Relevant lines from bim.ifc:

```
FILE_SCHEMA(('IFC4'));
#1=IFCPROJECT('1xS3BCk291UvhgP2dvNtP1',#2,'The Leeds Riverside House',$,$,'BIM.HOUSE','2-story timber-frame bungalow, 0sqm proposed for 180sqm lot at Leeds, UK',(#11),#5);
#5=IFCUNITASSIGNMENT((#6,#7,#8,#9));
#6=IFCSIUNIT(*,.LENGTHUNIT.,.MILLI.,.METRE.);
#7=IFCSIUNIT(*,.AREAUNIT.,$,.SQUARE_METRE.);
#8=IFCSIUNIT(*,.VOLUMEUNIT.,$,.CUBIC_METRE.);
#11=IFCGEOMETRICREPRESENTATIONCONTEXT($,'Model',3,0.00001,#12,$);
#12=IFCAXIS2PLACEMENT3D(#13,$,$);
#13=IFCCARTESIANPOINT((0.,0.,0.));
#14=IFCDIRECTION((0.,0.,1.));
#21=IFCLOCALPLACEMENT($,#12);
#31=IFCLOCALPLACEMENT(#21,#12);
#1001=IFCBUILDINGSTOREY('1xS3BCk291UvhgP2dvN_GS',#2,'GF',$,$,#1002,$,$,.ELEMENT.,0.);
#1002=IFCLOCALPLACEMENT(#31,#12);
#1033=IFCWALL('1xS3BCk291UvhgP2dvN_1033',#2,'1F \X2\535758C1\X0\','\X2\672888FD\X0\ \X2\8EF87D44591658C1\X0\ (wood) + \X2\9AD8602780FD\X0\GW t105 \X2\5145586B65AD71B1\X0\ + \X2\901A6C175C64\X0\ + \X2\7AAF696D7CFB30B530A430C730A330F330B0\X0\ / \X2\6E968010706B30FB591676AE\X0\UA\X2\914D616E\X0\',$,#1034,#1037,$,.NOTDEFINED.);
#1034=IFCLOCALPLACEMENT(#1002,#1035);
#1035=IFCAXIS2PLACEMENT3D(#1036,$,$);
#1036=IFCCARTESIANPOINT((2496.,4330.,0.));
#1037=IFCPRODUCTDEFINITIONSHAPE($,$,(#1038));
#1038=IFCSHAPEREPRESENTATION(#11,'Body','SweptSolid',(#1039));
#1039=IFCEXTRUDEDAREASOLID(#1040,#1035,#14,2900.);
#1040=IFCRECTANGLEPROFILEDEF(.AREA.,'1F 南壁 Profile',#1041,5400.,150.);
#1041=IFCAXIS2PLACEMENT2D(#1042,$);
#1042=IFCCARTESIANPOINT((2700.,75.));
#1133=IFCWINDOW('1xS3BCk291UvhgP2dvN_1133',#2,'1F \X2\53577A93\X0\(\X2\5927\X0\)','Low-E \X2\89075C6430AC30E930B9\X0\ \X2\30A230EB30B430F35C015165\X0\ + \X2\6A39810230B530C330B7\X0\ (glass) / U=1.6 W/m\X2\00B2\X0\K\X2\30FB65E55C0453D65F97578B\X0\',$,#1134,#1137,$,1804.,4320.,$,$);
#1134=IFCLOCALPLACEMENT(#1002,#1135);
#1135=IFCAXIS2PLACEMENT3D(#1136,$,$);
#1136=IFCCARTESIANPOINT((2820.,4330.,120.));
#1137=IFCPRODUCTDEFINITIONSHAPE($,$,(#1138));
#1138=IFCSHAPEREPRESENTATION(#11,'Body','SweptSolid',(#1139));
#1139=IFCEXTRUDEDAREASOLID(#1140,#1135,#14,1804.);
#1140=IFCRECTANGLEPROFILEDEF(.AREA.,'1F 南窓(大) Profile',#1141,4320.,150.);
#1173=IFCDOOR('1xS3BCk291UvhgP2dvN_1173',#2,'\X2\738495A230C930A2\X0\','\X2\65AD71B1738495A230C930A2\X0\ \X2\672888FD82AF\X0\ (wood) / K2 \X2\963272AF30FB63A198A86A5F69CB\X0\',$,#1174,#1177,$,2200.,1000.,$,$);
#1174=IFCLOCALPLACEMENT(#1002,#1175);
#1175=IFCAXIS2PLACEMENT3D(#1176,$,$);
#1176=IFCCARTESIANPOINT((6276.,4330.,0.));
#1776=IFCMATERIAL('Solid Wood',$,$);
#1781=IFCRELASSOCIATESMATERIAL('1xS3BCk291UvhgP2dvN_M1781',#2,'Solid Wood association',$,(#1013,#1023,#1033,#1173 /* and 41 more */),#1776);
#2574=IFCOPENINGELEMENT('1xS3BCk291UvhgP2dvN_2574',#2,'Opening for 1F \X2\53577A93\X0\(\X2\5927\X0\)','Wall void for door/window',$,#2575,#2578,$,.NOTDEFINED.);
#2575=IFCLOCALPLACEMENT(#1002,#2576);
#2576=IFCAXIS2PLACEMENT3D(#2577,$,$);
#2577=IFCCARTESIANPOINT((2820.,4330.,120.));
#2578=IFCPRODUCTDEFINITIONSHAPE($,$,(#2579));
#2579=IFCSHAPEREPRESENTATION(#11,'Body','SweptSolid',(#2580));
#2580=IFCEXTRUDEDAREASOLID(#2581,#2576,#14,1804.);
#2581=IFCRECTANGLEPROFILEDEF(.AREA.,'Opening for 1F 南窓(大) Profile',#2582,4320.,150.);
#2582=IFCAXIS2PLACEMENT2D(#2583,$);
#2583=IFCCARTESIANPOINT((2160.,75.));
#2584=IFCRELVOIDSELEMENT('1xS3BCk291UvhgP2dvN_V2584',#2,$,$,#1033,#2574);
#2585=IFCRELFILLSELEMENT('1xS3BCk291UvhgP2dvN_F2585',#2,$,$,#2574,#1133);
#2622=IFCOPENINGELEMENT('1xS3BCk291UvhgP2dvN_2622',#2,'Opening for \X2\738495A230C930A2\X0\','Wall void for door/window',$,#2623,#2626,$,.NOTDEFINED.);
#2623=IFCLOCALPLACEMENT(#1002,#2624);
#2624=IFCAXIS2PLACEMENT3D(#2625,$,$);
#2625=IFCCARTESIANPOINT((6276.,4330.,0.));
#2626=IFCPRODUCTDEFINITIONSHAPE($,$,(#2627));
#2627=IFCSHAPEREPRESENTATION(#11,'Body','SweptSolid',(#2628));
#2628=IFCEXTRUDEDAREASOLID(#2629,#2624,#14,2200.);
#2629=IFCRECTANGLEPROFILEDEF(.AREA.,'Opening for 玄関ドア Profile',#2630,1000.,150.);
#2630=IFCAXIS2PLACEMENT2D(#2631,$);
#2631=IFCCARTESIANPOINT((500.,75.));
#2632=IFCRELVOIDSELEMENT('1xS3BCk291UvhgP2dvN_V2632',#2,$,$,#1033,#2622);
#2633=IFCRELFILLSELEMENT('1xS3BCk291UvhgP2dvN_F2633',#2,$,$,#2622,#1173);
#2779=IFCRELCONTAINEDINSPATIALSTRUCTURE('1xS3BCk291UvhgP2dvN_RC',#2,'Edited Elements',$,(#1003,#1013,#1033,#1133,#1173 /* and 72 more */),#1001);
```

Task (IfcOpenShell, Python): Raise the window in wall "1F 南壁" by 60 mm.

```python
import numpy as np
import ifcopenshell
import ifcopenshell.api.geometry
import ifcopenshell.util.placement
import ifcopenshell.util.unit

model = ifcopenshell.open("bim.ifc")
unit_scale = ifcopenshell.util.unit.calculate_unit_scale(model)

window = model.by_guid("1xS3BCk291UvhgP2dvN_1133")
opening = window.FillsVoids[0].RelatingOpeningElement
dz = 0.06 / unit_scale

shift = np.array([0.0, 0.0, dz])
# The window is not placed relative to its opening, so move both.
for product in (opening, window):
    matrix = ifcopenshell.util.placement.get_local_placement(product.ObjectPlacement)
    matrix[:3, 3] += shift
    ifcopenshell.api.geometry.edit_object_placement(model, product=product, matrix=matrix, is_si=False)

print(f"moved by {dz * unit_scale:+.3f} m")

model.write("bim_edited.ifc")
```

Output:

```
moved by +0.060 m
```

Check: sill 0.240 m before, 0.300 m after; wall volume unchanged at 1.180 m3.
